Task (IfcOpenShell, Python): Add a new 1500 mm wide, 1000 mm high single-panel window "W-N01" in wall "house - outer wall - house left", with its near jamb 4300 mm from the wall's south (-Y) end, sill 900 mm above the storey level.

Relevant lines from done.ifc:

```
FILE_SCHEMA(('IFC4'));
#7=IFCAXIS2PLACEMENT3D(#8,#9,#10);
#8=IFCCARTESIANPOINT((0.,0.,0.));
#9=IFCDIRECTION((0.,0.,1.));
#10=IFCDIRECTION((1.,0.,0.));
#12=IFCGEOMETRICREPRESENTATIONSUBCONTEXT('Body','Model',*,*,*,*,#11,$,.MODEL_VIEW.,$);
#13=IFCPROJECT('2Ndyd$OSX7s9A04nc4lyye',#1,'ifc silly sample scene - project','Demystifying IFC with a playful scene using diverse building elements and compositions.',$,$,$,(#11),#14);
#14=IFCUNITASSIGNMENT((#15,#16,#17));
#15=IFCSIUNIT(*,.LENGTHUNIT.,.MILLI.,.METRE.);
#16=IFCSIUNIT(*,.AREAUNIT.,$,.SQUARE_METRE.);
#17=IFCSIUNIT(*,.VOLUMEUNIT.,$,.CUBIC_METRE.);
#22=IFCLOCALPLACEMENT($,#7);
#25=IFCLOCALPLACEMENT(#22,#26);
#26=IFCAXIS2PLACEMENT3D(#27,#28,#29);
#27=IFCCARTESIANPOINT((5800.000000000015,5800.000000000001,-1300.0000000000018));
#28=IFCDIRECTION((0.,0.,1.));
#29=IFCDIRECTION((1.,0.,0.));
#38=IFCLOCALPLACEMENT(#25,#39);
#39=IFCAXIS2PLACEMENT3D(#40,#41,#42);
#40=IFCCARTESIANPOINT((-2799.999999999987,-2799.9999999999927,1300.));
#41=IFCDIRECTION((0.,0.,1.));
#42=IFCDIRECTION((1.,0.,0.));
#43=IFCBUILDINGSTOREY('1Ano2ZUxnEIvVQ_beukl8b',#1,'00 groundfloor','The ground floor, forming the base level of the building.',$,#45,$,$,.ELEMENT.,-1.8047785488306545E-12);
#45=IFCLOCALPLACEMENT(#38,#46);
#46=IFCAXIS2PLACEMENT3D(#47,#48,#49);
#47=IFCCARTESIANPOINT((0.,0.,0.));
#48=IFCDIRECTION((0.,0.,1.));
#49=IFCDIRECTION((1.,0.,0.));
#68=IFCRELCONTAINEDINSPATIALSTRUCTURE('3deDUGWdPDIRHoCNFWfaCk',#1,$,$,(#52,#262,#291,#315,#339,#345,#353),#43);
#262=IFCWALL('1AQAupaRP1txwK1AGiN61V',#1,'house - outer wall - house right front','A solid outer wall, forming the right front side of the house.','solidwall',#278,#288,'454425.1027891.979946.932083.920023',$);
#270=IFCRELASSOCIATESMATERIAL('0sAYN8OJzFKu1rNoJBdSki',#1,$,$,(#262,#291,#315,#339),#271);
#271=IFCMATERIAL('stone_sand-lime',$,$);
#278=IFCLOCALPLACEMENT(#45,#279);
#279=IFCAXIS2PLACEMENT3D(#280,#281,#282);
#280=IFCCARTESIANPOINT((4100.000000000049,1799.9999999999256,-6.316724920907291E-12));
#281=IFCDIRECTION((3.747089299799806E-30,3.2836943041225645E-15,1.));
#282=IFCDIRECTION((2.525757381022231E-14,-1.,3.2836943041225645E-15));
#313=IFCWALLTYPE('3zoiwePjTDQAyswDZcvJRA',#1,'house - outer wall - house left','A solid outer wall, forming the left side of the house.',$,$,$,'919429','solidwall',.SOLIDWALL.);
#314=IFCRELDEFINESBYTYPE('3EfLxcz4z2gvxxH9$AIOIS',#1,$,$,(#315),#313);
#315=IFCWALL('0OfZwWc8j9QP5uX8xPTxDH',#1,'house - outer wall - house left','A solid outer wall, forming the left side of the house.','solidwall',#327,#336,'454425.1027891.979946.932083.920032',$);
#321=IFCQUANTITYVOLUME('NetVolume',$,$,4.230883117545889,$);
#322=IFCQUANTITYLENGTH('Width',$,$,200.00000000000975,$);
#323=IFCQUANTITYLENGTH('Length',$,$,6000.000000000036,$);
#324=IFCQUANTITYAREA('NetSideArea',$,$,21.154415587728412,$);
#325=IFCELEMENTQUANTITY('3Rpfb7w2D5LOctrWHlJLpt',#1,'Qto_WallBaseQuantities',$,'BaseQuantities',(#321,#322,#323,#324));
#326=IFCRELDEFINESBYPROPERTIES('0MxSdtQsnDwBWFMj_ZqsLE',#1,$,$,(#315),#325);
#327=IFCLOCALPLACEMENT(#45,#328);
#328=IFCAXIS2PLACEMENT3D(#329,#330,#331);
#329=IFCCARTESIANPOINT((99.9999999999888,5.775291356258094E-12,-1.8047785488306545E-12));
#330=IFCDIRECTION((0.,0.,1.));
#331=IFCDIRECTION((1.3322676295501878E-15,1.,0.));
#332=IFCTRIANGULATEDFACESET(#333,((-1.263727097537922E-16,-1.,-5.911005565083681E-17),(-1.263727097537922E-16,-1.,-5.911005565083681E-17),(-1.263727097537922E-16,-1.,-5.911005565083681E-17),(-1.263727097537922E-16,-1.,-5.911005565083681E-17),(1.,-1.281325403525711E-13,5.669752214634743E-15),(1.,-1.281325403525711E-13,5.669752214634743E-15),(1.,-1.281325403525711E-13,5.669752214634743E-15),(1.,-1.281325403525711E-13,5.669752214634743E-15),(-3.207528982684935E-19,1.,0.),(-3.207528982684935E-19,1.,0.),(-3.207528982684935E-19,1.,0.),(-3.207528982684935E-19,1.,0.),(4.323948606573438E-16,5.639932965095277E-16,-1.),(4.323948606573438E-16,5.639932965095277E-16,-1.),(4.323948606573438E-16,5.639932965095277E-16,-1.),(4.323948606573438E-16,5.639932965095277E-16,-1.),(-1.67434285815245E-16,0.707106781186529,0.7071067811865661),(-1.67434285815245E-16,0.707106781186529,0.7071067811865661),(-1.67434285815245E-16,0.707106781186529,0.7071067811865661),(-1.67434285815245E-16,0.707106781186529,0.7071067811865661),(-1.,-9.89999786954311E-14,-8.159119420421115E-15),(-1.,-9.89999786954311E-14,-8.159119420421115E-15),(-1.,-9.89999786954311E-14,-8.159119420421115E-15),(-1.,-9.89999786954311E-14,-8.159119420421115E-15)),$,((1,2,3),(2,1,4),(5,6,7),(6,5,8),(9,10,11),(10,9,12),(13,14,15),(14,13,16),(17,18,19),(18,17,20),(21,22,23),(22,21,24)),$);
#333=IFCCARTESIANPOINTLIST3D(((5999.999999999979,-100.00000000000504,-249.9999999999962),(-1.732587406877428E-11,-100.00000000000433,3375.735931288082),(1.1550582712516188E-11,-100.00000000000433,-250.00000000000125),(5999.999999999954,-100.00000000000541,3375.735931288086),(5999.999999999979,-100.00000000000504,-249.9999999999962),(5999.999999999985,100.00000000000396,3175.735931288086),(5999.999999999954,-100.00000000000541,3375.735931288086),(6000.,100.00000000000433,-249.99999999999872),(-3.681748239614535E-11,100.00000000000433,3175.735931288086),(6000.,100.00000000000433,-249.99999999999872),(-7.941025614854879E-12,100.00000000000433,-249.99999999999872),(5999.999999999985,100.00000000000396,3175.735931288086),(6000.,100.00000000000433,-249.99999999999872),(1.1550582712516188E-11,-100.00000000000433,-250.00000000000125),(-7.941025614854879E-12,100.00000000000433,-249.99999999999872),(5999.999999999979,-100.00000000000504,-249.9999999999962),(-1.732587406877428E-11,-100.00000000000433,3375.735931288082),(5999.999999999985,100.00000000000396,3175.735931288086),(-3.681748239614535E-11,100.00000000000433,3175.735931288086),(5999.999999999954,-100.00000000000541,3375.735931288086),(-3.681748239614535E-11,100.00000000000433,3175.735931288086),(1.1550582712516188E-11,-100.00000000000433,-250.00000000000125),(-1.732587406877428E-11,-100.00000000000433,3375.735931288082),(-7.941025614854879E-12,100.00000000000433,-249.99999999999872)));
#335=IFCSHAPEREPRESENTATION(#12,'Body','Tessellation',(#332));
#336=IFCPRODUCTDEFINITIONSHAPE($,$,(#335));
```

```python
import numpy as np
import ifcopenshell
import ifcopenshell.api.feature
import ifcopenshell.api.geometry
import ifcopenshell.api.pset
import ifcopenshell.api.root
import ifcopenshell.api.spatial
import ifcopenshell.geom
import ifcopenshell.util.element
import ifcopenshell.util.placement
import ifcopenshell.util.representation
import ifcopenshell.util.shape
import ifcopenshell.util.unit

model = ifcopenshell.open("done.ifc")
unit_scale = ifcopenshell.util.unit.calculate_unit_scale(model)
area_scale = ifcopenshell.util.unit.calculate_unit_scale(model, "AREAUNIT")
volume_scale = ifcopenshell.util.unit.calculate_unit_scale(model, "VOLUMEUNIT")
settings = ifcopenshell.geom.settings()


def volume(element):
    """Net volume in cubic metres, openings subtracted."""
    shape = ifcopenshell.geom.create_shape(settings, element)
    return ifcopenshell.util.shape.get_volume(shape.geometry)


wall = model.by_guid("0OfZwWc8j9QP5uX8xPTxDH")
storey = ifcopenshell.util.element.get_container(wall, ifc_class="IfcBuildingStorey")
context = ifcopenshell.util.representation.get_context(model, "Model", "Body", "MODEL_VIEW")
before = volume(wall)

width, height, from_end, sill = 1.5, 1, 4.3, 0.9  # metres

# The wall runs along its own X axis, and the end named is its -X end.
wall_shape = ifcopenshell.geom.create_shape(settings, wall)
x, y, z = ifcopenshell.util.shape.get_vertices(wall_shape.geometry).T
start = x.min() + from_end
face, thickness = float(y.min()), float(y.max() - y.min())
wall_matrix = ifcopenshell.util.placement.get_local_placement(wall.ObjectPlacement)
level = ifcopenshell.util.placement.get_local_placement(storey.ObjectPlacement)[2, 3]


def in_wall(x, y):
    """Placement at x, y metres in the wall's axes, at sill height."""
    matrix = wall_matrix.copy()
    matrix[:, 3] = wall_matrix @ np.array([x / unit_scale, y / unit_scale, 0.0, 1.0])
    matrix[2, 3] = level + sill / unit_scale
    return matrix


# Opening: a box that overshoots both wall faces by 50 mm.
opening = ifcopenshell.api.root.create_entity(model, ifc_class="IfcOpeningElement", predefined_type="OPENING")
box = ifcopenshell.api.geometry.add_wall_representation(
    model, context=context, length=width, height=height, thickness=thickness + 0.1
)
ifcopenshell.api.geometry.assign_representation(model, product=opening, representation=box)
ifcopenshell.api.geometry.edit_object_placement(model, product=opening, matrix=in_wall(start, face - 0.05), is_si=False)
ifcopenshell.api.feature.add_feature(model, feature=opening, element=wall)

window = ifcopenshell.api.root.create_entity(model, ifc_class="IfcWindow", name="W-N01", predefined_type="WINDOW")
window.OverallWidth, window.OverallHeight = width / unit_scale, height / unit_scale
window.PartitioningType = "SINGLE_PANEL"
body = ifcopenshell.api.geometry.add_window_representation(
    model,
    context=context,
    overall_width=window.OverallWidth,
    overall_height=window.OverallHeight,
    partition_type="SINGLE_PANEL",
)
ifcopenshell.api.geometry.assign_representation(model, product=window, representation=body)
ifcopenshell.api.spatial.assign_container(model, products=[window], relating_structure=storey)
ifcopenshell.api.feature.add_filling(model, opening=opening, element=window)

# Centre the window in the wall's thickness.
ifcopenshell.api.geometry.edit_object_placement(model, product=window, matrix=in_wall(start, face), is_si=False)
window_shape = ifcopenshell.geom.create_shape(settings, window)
depth = ifcopenshell.util.shape.get_vertices(window_shape.geometry)[:, 1]
offset = face + thickness / 2 - (depth.min() + depth.max()) / 2
ifcopenshell.api.geometry.edit_object_placement(model, product=window, matrix=in_wall(start, offset), is_si=False)

after = volume(wall)

# Update the wall's stored quantities.
qto = model.by_id(ifcopenshell.util.element.get_pset(wall, "Qto_WallBaseQuantities", should_inherit=False)["id"])
ifcopenshell.api.pset.edit_qto(model, qto=qto, properties={
    "NetVolume": after / volume_scale,
    "NetSideArea": after / thickness / area_scale,
})

print(f"wall volume {before:.3f} -> {after:.3f} m3")

model.write("done_v2.ifc")
```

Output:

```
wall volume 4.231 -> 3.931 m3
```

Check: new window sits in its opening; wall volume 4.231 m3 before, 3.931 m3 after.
